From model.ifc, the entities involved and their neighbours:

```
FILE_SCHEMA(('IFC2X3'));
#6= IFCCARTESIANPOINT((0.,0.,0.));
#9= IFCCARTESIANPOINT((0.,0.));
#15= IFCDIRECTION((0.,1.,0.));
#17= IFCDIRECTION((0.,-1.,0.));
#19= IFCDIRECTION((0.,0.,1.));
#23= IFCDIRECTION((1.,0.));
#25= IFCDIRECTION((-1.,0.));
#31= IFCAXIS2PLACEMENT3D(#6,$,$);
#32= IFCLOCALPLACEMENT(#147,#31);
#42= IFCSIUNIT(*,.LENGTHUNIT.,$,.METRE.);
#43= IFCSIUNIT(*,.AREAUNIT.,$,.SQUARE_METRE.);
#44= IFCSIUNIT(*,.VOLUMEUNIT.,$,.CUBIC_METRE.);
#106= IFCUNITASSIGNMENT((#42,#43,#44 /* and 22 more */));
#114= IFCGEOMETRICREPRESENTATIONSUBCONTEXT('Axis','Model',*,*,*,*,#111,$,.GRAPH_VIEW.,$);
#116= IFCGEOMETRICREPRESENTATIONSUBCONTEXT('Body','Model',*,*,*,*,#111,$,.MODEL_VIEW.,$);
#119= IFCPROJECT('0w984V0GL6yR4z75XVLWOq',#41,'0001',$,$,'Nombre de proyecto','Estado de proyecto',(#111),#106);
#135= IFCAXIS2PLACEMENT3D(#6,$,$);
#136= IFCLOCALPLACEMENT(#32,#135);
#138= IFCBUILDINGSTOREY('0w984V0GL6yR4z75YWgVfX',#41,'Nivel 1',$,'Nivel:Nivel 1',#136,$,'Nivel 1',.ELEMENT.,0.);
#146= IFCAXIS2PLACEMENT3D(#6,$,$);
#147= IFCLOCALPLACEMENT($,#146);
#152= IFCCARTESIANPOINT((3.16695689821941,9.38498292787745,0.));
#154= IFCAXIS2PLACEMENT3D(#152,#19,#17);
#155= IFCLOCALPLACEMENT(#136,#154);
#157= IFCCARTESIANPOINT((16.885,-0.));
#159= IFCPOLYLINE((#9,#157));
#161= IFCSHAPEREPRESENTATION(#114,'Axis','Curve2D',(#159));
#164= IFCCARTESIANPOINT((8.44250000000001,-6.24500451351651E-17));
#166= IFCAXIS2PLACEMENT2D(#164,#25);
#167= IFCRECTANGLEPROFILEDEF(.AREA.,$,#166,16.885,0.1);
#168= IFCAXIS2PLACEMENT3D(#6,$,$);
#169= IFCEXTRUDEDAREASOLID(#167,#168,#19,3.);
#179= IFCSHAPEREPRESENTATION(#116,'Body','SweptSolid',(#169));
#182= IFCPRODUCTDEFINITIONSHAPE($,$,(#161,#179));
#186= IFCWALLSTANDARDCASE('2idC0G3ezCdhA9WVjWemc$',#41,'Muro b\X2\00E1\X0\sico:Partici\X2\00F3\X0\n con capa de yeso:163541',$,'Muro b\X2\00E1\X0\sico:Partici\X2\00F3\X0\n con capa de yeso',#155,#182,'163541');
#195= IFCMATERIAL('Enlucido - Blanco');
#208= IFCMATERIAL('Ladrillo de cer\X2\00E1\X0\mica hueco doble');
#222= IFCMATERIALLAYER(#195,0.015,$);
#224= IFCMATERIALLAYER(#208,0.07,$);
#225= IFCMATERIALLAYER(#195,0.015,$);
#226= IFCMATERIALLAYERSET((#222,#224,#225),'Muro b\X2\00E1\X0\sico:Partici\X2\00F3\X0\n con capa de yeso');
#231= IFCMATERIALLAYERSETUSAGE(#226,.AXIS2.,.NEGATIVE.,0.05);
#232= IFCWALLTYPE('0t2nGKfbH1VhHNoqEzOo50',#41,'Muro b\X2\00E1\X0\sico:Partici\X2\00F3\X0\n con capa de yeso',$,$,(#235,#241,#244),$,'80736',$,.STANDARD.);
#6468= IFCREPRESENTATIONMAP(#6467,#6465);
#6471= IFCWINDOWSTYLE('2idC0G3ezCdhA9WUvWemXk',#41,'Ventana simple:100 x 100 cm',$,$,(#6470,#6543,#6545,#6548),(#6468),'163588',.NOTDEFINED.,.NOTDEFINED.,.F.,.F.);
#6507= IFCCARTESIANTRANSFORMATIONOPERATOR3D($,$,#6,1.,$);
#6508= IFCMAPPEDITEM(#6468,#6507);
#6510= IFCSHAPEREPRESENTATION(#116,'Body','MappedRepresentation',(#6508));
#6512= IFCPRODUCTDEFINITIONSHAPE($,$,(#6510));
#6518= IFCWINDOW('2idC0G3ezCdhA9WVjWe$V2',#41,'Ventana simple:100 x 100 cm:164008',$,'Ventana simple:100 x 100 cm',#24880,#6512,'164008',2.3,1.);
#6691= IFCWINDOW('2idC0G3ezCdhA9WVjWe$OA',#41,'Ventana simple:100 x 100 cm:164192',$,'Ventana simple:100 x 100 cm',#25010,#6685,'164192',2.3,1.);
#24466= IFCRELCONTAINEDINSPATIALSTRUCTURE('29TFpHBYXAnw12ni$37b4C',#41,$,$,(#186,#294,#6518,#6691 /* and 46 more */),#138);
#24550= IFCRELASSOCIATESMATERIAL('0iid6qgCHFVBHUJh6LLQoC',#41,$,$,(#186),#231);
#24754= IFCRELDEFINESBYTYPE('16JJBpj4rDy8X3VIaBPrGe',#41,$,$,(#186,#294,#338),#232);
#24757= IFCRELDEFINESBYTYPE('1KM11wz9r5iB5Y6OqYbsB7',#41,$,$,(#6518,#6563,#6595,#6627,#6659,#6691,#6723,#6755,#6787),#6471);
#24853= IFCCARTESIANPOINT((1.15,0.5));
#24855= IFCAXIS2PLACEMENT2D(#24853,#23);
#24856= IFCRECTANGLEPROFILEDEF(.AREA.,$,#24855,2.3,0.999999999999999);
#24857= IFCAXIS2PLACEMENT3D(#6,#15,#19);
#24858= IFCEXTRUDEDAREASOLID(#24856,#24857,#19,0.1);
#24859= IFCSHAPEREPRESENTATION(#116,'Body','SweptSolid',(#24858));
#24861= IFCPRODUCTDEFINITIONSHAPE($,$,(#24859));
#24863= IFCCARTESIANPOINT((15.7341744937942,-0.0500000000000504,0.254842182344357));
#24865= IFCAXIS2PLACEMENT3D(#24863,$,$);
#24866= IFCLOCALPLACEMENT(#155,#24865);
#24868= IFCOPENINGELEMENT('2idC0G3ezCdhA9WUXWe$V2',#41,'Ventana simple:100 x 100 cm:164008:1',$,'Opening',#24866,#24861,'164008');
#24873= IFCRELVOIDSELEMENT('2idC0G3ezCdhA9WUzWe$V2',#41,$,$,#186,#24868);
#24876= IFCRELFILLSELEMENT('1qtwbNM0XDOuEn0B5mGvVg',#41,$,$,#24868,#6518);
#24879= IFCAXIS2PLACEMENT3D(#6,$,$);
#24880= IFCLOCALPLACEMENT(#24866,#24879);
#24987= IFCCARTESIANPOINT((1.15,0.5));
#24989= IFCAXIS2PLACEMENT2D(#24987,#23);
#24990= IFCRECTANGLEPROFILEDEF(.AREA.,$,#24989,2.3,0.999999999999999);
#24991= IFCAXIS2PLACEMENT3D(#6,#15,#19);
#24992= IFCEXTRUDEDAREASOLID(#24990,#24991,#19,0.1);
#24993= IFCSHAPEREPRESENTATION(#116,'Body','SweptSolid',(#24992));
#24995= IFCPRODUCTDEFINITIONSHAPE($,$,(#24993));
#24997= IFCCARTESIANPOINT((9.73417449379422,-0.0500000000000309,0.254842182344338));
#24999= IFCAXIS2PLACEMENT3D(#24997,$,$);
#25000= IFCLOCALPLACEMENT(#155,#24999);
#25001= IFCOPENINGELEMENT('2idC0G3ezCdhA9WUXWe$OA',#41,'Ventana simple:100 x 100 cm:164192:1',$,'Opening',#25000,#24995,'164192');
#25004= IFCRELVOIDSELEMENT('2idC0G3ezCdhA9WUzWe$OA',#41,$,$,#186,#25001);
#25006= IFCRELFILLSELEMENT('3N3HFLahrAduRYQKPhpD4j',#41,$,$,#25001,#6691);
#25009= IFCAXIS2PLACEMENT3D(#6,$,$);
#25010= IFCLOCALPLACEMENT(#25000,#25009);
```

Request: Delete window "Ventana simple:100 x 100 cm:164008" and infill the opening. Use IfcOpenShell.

```python
import ifcopenshell
import ifcopenshell.api.feature
import ifcopenshell.api.root
import ifcopenshell.geom
import ifcopenshell.util.shape

model = ifcopenshell.open("model.ifc")
settings = ifcopenshell.geom.settings()


def volume(element):
    """Net volume in cubic metres, openings subtracted."""
    shape = ifcopenshell.geom.create_shape(settings, element)
    return ifcopenshell.util.shape.get_volume(shape.geometry)


window = model.by_guid("2idC0G3ezCdhA9WVjWe$V2")
opening = window.FillsVoids[0].RelatingOpeningElement
wall = opening.VoidsElements[0].RelatingBuildingElement
before = volume(wall)

ifcopenshell.api.root.remove_product(model, product=window)
ifcopenshell.api.feature.remove_feature(model, feature=opening)

after = volume(wall)

print(f"wall volume {before:.3f} -> {after:.3f} m3")

model.write("model_rev.ifc")
```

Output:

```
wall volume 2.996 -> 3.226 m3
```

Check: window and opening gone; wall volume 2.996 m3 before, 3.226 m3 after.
